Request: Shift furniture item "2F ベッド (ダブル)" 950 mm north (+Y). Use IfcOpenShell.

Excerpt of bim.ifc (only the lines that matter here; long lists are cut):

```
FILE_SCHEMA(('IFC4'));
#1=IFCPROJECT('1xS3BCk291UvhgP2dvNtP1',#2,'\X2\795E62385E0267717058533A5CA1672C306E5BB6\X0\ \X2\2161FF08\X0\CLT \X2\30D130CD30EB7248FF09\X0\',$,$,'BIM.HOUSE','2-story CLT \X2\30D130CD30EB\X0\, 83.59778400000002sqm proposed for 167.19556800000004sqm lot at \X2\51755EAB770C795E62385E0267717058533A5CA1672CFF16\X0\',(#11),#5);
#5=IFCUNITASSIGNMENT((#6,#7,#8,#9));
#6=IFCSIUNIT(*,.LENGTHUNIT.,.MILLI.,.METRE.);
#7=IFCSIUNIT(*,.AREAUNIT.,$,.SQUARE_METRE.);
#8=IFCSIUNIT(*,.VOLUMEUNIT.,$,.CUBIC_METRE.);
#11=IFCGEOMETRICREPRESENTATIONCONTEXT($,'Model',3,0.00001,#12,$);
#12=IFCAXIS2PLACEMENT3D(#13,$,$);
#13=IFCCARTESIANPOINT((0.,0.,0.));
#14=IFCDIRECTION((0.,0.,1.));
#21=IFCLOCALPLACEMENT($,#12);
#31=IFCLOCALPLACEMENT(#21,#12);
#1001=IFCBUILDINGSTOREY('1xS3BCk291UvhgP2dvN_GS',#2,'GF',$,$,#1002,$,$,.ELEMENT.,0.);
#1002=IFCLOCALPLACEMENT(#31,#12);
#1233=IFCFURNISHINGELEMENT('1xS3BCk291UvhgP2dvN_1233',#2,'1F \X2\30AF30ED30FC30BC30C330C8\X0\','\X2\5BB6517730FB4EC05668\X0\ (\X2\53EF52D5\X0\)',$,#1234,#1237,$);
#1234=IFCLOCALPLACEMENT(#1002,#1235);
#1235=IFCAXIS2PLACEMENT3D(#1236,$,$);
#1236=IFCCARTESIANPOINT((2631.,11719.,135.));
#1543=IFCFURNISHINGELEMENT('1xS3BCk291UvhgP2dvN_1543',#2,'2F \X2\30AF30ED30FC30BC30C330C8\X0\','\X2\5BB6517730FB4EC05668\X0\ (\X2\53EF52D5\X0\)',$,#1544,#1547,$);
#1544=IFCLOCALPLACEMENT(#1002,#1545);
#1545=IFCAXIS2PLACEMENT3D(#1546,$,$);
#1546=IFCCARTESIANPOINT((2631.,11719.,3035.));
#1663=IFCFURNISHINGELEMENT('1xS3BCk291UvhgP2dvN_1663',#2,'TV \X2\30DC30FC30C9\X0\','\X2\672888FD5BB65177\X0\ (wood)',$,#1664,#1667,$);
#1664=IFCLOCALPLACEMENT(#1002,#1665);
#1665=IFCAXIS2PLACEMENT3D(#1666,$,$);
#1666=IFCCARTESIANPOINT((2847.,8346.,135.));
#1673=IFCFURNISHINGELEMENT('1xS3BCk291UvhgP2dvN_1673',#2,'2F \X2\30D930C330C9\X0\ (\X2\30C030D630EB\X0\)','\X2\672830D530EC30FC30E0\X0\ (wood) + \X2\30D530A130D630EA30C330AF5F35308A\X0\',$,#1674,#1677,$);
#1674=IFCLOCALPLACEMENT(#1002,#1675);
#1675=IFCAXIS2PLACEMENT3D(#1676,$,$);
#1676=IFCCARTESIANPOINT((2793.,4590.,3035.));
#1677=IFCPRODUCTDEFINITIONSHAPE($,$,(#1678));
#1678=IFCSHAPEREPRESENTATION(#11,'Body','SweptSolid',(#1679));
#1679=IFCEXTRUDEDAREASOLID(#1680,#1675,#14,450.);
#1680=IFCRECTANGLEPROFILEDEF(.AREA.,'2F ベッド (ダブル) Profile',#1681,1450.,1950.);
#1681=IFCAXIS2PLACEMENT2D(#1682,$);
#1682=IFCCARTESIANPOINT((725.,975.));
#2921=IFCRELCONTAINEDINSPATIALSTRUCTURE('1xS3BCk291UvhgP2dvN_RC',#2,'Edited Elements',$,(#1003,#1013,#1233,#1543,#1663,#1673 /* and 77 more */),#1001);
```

```python
import ifcopenshell
import ifcopenshell.api.geometry
import ifcopenshell.util.placement
import ifcopenshell.util.unit

model = ifcopenshell.open("bim.ifc")
unit_scale = ifcopenshell.util.unit.calculate_unit_scale(model)

item = model.by_guid("1xS3BCk291UvhgP2dvN_1673")
matrix = ifcopenshell.util.placement.get_local_placement(item.ObjectPlacement)
matrix[1, 3] += 0.95 / unit_scale
ifcopenshell.api.geometry.edit_object_placement(model, product=item, matrix=matrix, is_si=False)

print(ifcopenshell.util.placement.get_local_placement(item.ObjectPlacement).round(3) + 0.0)

model.write("bim-out.ifc")
```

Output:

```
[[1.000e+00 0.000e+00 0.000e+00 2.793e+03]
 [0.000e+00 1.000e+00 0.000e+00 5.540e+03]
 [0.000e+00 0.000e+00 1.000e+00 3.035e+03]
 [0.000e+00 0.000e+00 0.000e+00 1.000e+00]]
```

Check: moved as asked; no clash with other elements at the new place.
